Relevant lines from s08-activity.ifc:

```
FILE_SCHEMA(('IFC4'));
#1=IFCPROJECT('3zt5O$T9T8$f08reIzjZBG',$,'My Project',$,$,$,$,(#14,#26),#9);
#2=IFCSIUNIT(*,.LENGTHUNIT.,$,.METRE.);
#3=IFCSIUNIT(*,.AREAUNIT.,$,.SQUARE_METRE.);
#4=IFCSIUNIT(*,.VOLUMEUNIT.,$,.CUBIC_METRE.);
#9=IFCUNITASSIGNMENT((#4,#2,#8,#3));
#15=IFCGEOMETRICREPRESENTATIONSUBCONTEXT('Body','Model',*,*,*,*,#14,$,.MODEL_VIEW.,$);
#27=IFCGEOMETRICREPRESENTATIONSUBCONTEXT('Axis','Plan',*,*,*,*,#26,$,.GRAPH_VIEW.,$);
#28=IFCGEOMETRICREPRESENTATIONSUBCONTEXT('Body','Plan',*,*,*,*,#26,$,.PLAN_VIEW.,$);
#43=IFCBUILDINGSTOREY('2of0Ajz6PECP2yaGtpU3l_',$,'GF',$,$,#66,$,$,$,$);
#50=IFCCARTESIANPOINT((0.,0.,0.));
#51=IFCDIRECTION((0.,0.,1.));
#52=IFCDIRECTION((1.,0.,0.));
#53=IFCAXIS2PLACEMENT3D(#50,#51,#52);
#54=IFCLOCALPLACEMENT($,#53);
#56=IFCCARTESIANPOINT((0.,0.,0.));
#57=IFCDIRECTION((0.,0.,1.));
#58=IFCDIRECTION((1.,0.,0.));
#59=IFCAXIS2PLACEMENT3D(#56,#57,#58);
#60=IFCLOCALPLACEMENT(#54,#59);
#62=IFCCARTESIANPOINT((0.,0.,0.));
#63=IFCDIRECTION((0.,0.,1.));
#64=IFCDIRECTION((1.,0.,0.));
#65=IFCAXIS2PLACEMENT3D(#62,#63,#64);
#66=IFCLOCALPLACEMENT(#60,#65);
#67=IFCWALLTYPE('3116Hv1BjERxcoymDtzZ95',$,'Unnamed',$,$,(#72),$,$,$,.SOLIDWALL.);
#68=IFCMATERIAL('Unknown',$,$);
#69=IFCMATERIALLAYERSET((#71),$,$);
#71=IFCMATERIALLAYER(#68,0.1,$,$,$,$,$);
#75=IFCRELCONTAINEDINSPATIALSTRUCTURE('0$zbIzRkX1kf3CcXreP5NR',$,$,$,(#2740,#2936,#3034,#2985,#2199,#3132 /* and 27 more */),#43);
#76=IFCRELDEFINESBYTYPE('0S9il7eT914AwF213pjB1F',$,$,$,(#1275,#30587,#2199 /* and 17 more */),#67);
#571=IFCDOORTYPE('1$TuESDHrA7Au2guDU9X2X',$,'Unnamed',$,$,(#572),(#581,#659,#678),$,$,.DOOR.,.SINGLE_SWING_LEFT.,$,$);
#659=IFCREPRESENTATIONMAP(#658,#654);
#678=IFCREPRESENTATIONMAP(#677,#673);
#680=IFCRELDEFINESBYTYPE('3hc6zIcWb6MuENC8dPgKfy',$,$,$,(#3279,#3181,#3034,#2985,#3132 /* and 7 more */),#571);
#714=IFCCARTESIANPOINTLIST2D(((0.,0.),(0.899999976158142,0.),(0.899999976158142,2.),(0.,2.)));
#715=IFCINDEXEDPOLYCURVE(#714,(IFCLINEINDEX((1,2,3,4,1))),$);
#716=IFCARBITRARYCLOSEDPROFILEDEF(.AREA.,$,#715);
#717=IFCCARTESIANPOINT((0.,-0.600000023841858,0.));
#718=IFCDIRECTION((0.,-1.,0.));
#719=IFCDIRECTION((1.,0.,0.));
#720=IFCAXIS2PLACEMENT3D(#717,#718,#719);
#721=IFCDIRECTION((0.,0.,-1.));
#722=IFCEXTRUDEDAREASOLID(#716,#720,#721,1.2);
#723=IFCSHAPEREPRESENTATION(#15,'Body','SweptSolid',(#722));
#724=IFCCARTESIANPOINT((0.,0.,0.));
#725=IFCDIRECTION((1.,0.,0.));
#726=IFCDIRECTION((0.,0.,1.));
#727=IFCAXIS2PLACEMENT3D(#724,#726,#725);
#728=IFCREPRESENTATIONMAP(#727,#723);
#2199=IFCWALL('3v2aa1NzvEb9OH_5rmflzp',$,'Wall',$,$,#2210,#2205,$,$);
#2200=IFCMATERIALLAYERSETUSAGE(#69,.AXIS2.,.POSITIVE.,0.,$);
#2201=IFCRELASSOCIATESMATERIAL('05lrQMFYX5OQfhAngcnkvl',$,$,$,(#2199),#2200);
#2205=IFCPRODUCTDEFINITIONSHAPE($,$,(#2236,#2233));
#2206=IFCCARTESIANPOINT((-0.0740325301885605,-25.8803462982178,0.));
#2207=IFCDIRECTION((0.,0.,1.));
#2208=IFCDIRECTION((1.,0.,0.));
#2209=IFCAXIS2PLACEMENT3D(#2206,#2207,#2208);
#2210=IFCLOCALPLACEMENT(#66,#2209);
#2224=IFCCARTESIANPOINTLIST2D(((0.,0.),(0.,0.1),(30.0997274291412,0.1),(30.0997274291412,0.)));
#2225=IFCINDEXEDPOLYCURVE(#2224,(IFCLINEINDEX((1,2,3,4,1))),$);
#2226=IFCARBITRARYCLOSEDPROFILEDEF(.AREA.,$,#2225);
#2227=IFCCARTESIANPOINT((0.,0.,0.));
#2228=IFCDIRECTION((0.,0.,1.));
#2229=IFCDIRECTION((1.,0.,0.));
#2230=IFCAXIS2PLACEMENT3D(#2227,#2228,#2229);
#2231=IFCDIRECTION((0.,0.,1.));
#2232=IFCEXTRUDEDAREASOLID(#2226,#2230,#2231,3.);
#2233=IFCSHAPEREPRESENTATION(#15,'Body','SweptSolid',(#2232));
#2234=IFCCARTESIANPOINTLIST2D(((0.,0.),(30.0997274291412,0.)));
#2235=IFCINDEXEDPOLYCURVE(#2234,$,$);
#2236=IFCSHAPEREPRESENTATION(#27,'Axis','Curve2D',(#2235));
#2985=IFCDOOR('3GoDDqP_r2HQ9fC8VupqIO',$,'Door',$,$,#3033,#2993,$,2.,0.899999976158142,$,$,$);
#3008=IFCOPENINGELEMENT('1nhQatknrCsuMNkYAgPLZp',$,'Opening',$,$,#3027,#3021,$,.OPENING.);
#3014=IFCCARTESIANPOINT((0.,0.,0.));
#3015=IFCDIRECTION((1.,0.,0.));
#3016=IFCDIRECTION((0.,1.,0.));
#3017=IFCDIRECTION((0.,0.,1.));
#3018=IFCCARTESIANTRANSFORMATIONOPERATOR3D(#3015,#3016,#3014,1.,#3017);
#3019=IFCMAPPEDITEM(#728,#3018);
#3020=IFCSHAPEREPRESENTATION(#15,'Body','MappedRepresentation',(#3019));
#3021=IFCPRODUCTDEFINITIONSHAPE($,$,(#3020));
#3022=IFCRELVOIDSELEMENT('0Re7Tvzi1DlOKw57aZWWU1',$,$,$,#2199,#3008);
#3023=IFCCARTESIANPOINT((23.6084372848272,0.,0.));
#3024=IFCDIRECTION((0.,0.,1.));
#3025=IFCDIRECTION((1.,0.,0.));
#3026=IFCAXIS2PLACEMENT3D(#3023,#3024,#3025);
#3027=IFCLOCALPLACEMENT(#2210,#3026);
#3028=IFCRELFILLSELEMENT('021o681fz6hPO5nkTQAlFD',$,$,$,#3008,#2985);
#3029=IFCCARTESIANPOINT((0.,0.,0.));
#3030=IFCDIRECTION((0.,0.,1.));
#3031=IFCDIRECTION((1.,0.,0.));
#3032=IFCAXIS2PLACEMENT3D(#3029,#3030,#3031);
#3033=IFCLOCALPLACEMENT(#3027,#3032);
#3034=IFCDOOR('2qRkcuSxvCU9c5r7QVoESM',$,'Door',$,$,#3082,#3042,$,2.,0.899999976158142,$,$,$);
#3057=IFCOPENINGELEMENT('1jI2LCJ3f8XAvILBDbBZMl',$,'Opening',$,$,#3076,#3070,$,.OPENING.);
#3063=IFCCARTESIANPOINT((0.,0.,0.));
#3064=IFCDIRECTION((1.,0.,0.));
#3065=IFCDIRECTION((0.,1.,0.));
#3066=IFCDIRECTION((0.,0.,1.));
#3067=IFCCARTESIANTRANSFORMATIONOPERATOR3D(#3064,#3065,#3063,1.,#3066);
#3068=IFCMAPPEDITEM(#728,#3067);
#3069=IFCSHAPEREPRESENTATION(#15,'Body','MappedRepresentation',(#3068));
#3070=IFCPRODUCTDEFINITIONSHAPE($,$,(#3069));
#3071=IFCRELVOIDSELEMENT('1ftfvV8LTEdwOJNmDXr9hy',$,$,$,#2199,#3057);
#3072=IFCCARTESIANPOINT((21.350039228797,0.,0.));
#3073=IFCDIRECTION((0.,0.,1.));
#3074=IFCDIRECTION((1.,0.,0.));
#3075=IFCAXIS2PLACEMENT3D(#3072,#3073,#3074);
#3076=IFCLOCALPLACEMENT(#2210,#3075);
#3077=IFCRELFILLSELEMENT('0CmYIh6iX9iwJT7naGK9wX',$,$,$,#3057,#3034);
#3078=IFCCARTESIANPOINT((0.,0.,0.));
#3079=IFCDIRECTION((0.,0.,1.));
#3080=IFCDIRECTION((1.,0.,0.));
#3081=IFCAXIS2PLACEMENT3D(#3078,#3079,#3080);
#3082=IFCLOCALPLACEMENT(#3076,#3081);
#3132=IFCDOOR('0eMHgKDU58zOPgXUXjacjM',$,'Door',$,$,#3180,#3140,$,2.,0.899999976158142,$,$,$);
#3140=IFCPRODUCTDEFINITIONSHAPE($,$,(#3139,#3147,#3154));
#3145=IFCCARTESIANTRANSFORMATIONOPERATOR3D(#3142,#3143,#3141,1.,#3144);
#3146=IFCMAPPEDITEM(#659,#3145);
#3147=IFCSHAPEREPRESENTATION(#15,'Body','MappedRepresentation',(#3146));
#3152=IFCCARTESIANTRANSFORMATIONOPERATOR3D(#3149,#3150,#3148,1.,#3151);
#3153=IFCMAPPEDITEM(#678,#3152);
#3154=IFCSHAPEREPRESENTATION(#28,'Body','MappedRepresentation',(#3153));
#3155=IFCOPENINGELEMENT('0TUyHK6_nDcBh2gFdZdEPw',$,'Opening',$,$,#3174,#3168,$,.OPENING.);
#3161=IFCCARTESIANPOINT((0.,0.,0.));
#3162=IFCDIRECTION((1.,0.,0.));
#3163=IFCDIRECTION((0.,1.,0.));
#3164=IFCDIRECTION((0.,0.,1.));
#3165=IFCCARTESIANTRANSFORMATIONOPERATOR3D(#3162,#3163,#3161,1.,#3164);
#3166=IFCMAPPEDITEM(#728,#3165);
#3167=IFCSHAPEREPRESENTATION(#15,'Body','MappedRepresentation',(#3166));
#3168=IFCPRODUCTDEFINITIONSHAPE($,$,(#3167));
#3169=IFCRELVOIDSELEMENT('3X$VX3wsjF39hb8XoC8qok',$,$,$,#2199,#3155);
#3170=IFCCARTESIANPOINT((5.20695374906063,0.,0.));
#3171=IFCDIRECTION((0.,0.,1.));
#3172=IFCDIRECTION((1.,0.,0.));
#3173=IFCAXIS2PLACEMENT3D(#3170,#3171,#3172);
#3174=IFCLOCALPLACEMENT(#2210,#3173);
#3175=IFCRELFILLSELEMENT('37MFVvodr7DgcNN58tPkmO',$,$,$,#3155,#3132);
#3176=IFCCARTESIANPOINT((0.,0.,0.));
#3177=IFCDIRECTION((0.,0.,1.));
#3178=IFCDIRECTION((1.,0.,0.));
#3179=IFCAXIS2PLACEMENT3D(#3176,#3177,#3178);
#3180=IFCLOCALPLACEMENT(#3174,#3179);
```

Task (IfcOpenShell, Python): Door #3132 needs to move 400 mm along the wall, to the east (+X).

```python
import ifcopenshell
import ifcopenshell.api.geometry
import ifcopenshell.util.placement

model = ifcopenshell.open("s08-activity.ifc")

door = model.by_guid("0eMHgKDU58zOPgXUXjacjM")
opening = door.FillsVoids[0].RelatingOpeningElement
wall = opening.VoidsElements[0].RelatingBuildingElement

wall_matrix = ifcopenshell.util.placement.get_local_placement(wall.ObjectPlacement)
shift = wall_matrix[:3, 0] * 0.4
before = ifcopenshell.util.placement.get_local_placement(door.ObjectPlacement)[:3, 3].copy()

# The door is placed relative to its opening, so it follows when the opening moves.
matrix = ifcopenshell.util.placement.get_local_placement(opening.ObjectPlacement)
matrix[:3, 3] += shift
ifcopenshell.api.geometry.edit_object_placement(
    model, product=opening, matrix=matrix, is_si=False, should_transform_children=True
)

after = ifcopenshell.util.placement.get_local_placement(door.ObjectPlacement)[:3, 3]
print("door moved by", (after - before).round(3) + 0.0)

model.write("s08-activity_updated.ifc")
```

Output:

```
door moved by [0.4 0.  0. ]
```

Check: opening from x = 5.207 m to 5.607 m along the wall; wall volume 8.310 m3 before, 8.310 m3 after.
